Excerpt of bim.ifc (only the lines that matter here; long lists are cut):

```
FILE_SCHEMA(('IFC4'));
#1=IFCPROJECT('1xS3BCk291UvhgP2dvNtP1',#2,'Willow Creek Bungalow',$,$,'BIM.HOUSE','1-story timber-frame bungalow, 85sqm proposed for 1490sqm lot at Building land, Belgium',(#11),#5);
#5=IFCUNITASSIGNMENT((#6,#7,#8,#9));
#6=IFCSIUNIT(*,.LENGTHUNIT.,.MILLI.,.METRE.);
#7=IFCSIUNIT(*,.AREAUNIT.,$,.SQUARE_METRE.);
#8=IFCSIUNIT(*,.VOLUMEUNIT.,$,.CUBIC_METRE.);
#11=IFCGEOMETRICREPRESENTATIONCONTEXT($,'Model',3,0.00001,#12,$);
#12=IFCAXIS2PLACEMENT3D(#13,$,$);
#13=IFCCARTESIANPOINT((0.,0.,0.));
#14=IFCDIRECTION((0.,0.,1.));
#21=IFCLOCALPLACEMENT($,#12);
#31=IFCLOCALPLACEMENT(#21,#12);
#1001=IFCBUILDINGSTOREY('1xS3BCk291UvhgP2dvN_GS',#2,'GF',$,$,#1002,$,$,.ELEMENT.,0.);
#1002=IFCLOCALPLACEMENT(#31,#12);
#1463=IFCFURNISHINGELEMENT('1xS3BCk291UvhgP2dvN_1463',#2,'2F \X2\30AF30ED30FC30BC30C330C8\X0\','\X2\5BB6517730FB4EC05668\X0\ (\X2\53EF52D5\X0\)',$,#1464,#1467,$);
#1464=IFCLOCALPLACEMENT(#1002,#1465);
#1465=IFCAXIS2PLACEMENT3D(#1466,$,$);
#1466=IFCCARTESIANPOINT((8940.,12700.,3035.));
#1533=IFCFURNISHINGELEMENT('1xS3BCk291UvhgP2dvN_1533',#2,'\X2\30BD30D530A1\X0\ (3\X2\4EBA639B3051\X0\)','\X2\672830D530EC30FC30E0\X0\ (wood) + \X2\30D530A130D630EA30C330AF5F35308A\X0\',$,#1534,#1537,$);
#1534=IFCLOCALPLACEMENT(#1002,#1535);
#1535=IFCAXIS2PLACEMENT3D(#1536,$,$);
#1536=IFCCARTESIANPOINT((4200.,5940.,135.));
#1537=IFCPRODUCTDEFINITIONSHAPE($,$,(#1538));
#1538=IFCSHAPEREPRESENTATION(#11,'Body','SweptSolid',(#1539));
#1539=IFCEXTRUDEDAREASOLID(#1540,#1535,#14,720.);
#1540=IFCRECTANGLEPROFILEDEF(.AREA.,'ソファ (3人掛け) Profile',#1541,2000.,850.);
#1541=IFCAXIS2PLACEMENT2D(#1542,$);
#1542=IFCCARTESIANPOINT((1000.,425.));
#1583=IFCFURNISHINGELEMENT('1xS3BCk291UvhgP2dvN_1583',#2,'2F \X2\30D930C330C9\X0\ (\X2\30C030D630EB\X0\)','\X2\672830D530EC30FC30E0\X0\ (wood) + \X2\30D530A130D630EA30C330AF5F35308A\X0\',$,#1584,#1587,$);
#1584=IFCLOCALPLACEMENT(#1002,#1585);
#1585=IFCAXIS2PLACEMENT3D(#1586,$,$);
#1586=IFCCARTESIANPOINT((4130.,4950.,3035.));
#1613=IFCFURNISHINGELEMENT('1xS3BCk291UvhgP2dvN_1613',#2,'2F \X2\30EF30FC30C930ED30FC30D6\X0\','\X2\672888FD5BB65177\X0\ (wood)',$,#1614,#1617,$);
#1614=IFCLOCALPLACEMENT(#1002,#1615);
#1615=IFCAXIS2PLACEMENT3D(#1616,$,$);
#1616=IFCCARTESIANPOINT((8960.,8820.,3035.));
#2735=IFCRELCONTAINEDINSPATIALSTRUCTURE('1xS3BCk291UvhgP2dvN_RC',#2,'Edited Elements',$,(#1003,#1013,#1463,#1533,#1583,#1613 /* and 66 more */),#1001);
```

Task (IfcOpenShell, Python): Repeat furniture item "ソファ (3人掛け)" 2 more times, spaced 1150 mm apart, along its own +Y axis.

```python
import ifcopenshell
import ifcopenshell.api.geometry
import ifcopenshell.api.root
import ifcopenshell.util.element
import ifcopenshell.util.placement

model = ifcopenshell.open("bim.ifc")


def reuse_history(source, copy):
    """copy_class also copies each property set's owner history, people and application; keep the originals."""
    for rel in copy.IsDefinedBy:
        if rel.is_a("IfcRelDefinesByProperties") and (history := rel.RelatingPropertyDefinition.OwnerHistory):
            rel.RelatingPropertyDefinition.OwnerHistory = source.OwnerHistory
            ifcopenshell.util.element.remove_deep2(model, history)


source = model.by_guid("1xS3BCk291UvhgP2dvN_1533")
base = ifcopenshell.util.placement.get_local_placement(source.ObjectPlacement)
step = base[:3, 1] * 1150.0

for i in range(1, 3):
    copy = ifcopenshell.api.root.copy_class(model, product=source)
    copy.Representation = ifcopenshell.util.element.copy_deep(
        model, source.Representation, exclude=["IfcGeometricRepresentationContext", "IfcRepresentationMap"]
    )
    reuse_history(source, copy)
    matrix = base.copy()
    matrix[:3, 3] += i * step
    print("added at", matrix[:3, 3].round(3) + 0.0)
    ifcopenshell.api.geometry.edit_object_placement(model, product=copy, matrix=matrix, is_si=False)

model.write("bim_updated.ifc")
```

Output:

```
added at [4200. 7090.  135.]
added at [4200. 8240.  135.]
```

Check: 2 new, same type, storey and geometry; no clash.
